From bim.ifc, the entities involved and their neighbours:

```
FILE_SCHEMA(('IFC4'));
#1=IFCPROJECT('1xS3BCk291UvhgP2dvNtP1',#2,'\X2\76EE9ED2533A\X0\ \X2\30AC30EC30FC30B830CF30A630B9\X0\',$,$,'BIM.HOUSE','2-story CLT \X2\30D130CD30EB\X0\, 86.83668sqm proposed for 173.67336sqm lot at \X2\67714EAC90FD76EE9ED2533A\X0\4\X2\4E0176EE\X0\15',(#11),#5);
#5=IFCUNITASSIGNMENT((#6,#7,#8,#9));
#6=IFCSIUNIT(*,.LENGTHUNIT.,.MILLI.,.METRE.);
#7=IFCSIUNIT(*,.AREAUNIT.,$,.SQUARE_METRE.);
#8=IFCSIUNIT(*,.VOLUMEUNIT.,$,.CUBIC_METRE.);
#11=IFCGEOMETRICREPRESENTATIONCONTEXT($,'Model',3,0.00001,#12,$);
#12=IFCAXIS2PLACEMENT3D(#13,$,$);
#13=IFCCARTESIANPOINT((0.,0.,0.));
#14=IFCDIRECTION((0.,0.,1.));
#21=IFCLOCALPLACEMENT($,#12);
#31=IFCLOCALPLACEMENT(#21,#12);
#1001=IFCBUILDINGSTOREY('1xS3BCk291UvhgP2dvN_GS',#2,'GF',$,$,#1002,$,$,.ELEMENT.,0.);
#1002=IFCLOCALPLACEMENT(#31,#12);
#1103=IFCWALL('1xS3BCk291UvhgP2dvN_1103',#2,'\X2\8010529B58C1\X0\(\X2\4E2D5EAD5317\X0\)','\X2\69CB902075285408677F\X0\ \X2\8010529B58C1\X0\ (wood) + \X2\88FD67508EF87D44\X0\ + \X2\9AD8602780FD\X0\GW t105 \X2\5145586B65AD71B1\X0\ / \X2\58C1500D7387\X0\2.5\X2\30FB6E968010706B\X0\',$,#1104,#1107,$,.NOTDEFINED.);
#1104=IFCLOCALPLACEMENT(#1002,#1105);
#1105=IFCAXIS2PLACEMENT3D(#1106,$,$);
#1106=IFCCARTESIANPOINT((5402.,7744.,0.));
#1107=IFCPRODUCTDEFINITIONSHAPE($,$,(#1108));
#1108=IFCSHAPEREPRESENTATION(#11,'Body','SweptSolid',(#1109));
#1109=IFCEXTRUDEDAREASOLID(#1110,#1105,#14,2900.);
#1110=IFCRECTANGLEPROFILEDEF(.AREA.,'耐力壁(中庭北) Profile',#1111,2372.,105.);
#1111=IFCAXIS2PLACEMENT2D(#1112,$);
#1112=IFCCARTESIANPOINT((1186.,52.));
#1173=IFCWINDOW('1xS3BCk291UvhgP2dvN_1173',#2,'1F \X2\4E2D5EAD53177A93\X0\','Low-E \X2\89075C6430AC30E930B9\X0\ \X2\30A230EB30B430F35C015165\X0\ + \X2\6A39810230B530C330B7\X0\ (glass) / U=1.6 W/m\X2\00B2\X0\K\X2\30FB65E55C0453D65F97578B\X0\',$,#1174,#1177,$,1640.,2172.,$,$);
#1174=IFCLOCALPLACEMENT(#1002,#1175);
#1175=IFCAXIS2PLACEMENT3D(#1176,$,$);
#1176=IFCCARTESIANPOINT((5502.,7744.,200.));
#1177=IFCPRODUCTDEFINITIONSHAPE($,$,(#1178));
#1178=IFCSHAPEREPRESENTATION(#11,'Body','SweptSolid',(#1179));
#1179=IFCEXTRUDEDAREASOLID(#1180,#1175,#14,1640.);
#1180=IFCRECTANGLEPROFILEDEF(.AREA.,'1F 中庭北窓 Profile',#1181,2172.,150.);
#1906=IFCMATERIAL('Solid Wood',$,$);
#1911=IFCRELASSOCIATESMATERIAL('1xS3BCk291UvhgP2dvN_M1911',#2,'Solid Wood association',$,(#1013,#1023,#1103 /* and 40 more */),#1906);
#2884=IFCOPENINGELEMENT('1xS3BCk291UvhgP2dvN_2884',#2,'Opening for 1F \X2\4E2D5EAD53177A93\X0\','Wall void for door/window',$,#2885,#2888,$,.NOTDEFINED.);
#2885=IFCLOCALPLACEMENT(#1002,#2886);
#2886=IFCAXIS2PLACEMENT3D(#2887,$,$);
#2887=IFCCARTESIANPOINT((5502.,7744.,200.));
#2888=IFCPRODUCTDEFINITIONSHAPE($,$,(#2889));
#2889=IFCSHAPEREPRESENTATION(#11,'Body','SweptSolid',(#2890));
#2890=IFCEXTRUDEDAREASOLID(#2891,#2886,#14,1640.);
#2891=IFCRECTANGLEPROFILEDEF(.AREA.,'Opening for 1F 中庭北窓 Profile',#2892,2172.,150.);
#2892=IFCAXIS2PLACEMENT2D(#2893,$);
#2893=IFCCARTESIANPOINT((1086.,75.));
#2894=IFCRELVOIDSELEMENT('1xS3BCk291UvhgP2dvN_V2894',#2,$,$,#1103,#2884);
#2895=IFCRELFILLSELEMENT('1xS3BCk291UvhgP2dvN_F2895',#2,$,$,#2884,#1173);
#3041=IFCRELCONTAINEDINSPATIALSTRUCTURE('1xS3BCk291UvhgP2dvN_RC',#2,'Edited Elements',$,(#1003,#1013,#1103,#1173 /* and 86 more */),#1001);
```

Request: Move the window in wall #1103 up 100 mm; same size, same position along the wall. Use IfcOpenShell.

```python
import numpy as np
import ifcopenshell
import ifcopenshell.api.geometry
import ifcopenshell.util.placement
import ifcopenshell.util.unit

model = ifcopenshell.open("bim.ifc")
unit_scale = ifcopenshell.util.unit.calculate_unit_scale(model)

window = model.by_guid("1xS3BCk291UvhgP2dvN_1173")
opening = window.FillsVoids[0].RelatingOpeningElement
dz = 100.0

shift = np.array([0.0, 0.0, dz])
# The window is not placed relative to its opening, so move both.
for product in (opening, window):
    matrix = ifcopenshell.util.placement.get_local_placement(product.ObjectPlacement)
    matrix[:3, 3] += shift
    ifcopenshell.api.geometry.edit_object_placement(model, product=product, matrix=matrix, is_si=False)

print(f"moved by {dz * unit_scale:+.3f} m")

model.write("bim_v2.ifc")
```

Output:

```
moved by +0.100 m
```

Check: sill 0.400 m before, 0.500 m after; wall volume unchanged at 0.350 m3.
